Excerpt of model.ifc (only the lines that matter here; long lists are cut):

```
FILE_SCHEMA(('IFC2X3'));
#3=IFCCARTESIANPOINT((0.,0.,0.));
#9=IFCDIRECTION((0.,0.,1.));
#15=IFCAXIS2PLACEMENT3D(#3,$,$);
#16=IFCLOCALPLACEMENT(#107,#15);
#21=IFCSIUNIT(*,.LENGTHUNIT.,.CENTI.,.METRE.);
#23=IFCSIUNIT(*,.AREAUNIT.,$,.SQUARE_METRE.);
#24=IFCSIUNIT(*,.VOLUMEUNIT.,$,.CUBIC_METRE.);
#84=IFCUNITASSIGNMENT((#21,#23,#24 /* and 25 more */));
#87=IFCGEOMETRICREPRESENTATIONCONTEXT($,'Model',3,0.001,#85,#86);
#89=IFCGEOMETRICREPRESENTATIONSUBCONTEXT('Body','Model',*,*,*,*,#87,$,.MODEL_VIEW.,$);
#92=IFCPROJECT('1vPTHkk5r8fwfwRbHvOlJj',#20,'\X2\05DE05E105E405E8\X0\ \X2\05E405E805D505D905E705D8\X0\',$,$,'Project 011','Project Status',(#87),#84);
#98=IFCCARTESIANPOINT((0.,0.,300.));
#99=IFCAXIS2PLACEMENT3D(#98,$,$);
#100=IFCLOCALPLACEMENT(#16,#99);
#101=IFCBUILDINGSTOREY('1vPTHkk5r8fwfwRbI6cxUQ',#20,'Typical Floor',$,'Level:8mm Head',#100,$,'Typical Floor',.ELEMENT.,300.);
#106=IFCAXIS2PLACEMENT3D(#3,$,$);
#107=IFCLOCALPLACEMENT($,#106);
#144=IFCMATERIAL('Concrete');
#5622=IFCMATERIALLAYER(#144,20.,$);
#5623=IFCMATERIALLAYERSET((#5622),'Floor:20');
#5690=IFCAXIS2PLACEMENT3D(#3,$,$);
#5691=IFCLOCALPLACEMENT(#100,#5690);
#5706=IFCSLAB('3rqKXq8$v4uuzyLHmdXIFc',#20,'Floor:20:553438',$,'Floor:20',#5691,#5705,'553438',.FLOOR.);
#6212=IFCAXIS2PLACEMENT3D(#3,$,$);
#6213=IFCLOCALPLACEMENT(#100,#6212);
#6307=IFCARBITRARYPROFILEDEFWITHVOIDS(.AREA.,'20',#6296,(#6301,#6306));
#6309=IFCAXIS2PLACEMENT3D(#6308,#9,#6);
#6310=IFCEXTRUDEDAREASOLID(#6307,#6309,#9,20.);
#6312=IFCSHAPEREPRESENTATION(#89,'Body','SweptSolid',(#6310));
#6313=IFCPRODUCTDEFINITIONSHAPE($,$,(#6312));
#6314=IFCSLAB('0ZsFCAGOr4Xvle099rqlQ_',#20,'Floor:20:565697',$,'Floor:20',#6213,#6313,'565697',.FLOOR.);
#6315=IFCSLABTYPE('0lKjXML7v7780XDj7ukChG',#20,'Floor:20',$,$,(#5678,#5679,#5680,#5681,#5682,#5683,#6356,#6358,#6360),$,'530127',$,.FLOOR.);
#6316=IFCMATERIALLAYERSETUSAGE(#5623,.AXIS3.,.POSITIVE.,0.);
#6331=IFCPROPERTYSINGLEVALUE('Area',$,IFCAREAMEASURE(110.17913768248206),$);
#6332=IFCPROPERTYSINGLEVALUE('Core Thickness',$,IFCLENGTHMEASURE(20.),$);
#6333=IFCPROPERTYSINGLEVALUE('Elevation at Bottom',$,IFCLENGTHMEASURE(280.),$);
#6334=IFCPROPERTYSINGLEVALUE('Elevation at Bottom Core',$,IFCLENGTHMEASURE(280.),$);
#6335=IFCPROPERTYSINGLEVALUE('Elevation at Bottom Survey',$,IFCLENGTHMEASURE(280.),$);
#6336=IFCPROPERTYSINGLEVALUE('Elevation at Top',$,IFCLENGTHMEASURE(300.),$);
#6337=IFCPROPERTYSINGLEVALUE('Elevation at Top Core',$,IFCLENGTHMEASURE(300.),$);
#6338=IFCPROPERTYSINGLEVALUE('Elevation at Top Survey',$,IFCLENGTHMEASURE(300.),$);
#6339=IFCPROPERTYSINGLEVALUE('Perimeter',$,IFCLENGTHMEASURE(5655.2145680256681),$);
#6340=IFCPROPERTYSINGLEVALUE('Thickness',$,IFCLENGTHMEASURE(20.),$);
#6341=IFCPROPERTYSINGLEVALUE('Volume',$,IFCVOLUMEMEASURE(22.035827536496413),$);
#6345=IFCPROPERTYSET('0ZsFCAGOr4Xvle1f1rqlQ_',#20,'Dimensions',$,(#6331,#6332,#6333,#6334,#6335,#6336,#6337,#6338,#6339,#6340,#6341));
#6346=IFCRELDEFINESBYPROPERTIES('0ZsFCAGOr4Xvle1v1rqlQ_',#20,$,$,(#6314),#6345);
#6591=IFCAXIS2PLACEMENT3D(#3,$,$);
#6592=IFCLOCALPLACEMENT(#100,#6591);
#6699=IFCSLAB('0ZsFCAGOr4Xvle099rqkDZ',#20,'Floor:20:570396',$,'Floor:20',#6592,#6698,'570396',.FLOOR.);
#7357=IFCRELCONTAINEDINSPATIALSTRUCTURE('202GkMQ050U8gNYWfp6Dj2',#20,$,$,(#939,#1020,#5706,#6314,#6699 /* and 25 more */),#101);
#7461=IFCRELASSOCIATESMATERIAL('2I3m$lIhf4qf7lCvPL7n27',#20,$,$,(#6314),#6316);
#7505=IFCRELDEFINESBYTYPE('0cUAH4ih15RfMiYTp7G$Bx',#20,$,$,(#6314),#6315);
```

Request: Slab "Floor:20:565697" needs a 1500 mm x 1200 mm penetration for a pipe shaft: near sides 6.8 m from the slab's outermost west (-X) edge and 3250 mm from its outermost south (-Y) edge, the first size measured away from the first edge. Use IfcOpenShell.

```python
import numpy as np
import ifcopenshell
import ifcopenshell.api.feature
import ifcopenshell.api.geometry
import ifcopenshell.api.pset
import ifcopenshell.api.root
import ifcopenshell.geom
import ifcopenshell.util.element
import ifcopenshell.util.placement
import ifcopenshell.util.representation
import ifcopenshell.util.shape
import ifcopenshell.util.unit

model = ifcopenshell.open("model.ifc")
unit_scale = ifcopenshell.util.unit.calculate_unit_scale(model)
area_scale = ifcopenshell.util.unit.calculate_unit_scale(model, "AREAUNIT")
volume_scale = ifcopenshell.util.unit.calculate_unit_scale(model, "VOLUMEUNIT")
settings = ifcopenshell.geom.settings()


def volume(element):
    """Net volume in cubic metres, openings subtracted."""
    shape = ifcopenshell.geom.create_shape(settings, element)
    return ifcopenshell.util.shape.get_volume(shape.geometry)


slab = model.by_guid("0ZsFCAGOr4Xvle099rqlQ_")
before = volume(slab)

# Extent in the slab's own axes, in metres. The edges named are its -X and -Y sides.
slab_shape = ifcopenshell.geom.create_shape(settings, slab)
vertices = ifcopenshell.util.shape.get_vertices(slab_shape.geometry)
x_min, y_min, bottom = vertices.min(axis=0)
top = vertices[:, 2].max()

opening = ifcopenshell.api.root.create_entity(model, ifc_class="IfcOpeningElement", name="Pipe shaft opening")
context = ifcopenshell.util.representation.get_context(model, "Model", "Body", "MODEL_VIEW")
width, depth = 1.5, 1.2
outline = [(0.0, 0.0), (width, 0.0), (width, depth), (0.0, depth), (0.0, 0.0)]
# Overshoot both faces by 50 mm so the cut is clean.
shape = ifcopenshell.api.geometry.add_slab_representation(
    model, context=context, depth=top - bottom + 0.1, polyline=outline
)
ifcopenshell.api.geometry.assign_representation(model, product=opening, representation=shape)

matrix = ifcopenshell.util.placement.get_local_placement(slab.ObjectPlacement)
matrix[:, 3] = matrix @ np.append(np.array([x_min + 6.8, y_min + 3.25, bottom - 0.05]) / unit_scale, 1.0)
ifcopenshell.api.geometry.edit_object_placement(model, product=opening, matrix=matrix, is_si=False)
ifcopenshell.api.feature.add_feature(model, feature=opening, element=slab)

after = volume(slab)

# Update the slab's stored quantities.
pset = model.by_id(ifcopenshell.util.element.get_pset(slab, "Dimensions", should_inherit=False)["id"])
ifcopenshell.api.pset.edit_pset(model, pset=pset, properties={
    "Area": model.create_entity("IfcAreaMeasure", after / (top - bottom) / area_scale),
    "Volume": model.create_entity("IfcVolumeMeasure", after / volume_scale),
})

print(f"slab volume {before:.3f} -> {after:.3f} m3")

model.write("model_updated.ifc")
```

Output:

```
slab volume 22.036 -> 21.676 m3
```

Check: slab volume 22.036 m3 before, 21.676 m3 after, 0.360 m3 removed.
